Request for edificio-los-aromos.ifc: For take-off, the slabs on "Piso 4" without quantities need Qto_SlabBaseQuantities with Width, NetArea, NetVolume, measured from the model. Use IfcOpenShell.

First a look at what the model holds.

```python
import ifcopenshell
import ifcopenshell.util.element
import ifcopenshell.util.unit

model = ifcopenshell.open("edificio-los-aromos.ifc")
print(model.schema)
for unit_type in ("LENGTHUNIT", "AREAUNIT", "VOLUMEUNIT"):
    print(unit_type, ifcopenshell.util.unit.calculate_unit_scale(model, unit_type))
storey = next(s for s in model.by_type("IfcBuildingStorey") if s.Name == "Piso 4")
slabs = [e for e in ifcopenshell.util.element.get_decomposition(storey) if e.is_a("IfcSlab")]
for e in sorted(slabs, key=lambda e: e.id()):
    print(e.id(), e.is_a(), e.Name, list(ifcopenshell.util.element.get_psets(e, qtos_only=True)), sep=" | ")
```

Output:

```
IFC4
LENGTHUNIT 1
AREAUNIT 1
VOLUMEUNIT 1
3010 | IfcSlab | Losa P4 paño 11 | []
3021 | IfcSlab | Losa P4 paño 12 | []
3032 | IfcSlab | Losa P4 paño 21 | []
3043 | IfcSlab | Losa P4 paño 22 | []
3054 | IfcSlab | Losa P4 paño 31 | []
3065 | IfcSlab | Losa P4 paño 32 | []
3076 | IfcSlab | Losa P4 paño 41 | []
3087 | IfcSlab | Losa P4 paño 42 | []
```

```python
import ifcopenshell
import ifcopenshell.api.pset
import ifcopenshell.geom
import ifcopenshell.util.element
import ifcopenshell.util.shape
import ifcopenshell.util.unit

model = ifcopenshell.open("edificio-los-aromos.ifc")
unit_scale = ifcopenshell.util.unit.calculate_unit_scale(model)
area_scale = ifcopenshell.util.unit.calculate_unit_scale(model, "AREAUNIT")
volume_scale = ifcopenshell.util.unit.calculate_unit_scale(model, "VOLUMEUNIT")
settings = ifcopenshell.geom.settings()

storey = next(s for s in model.by_type("IfcBuildingStorey") if s.Name == "Piso 4")
slabs = [e for e in ifcopenshell.util.element.get_decomposition(storey) if e.is_a("IfcSlab")]

for e in sorted(slabs, key=lambda e: e.id()):
    if ifcopenshell.util.element.get_psets(e, qtos_only=True, should_inherit=False):
        continue
    # Geometry comes back in metres, in the element's own axes.
    shape = ifcopenshell.geom.create_shape(settings, e)
    values = {
        "Width": ifcopenshell.util.shape.get_z(shape.geometry) / unit_scale,
        "NetArea": ifcopenshell.util.shape.get_footprint_area(shape.geometry) / area_scale,
        "NetVolume": ifcopenshell.util.shape.get_volume(shape.geometry) / volume_scale,
    }
    qto = ifcopenshell.api.pset.add_qto(model, product=e, name="Qto_SlabBaseQuantities")
    ifcopenshell.api.pset.edit_qto(model, qto=qto, properties=values)
    print(e.id(), {k: round(v, 3) for k, v in values.items()})

model.write("edificio-los-aromos-out.ifc")
```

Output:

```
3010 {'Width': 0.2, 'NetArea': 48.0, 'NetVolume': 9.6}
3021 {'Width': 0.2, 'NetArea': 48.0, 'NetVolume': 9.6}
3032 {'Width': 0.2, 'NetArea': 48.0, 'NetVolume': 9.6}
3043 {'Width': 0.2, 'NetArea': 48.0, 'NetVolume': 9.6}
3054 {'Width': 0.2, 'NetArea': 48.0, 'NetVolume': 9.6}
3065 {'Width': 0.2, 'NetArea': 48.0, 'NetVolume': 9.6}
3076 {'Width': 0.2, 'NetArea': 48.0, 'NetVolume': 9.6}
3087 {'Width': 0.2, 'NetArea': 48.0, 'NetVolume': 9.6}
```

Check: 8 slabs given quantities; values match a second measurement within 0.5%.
